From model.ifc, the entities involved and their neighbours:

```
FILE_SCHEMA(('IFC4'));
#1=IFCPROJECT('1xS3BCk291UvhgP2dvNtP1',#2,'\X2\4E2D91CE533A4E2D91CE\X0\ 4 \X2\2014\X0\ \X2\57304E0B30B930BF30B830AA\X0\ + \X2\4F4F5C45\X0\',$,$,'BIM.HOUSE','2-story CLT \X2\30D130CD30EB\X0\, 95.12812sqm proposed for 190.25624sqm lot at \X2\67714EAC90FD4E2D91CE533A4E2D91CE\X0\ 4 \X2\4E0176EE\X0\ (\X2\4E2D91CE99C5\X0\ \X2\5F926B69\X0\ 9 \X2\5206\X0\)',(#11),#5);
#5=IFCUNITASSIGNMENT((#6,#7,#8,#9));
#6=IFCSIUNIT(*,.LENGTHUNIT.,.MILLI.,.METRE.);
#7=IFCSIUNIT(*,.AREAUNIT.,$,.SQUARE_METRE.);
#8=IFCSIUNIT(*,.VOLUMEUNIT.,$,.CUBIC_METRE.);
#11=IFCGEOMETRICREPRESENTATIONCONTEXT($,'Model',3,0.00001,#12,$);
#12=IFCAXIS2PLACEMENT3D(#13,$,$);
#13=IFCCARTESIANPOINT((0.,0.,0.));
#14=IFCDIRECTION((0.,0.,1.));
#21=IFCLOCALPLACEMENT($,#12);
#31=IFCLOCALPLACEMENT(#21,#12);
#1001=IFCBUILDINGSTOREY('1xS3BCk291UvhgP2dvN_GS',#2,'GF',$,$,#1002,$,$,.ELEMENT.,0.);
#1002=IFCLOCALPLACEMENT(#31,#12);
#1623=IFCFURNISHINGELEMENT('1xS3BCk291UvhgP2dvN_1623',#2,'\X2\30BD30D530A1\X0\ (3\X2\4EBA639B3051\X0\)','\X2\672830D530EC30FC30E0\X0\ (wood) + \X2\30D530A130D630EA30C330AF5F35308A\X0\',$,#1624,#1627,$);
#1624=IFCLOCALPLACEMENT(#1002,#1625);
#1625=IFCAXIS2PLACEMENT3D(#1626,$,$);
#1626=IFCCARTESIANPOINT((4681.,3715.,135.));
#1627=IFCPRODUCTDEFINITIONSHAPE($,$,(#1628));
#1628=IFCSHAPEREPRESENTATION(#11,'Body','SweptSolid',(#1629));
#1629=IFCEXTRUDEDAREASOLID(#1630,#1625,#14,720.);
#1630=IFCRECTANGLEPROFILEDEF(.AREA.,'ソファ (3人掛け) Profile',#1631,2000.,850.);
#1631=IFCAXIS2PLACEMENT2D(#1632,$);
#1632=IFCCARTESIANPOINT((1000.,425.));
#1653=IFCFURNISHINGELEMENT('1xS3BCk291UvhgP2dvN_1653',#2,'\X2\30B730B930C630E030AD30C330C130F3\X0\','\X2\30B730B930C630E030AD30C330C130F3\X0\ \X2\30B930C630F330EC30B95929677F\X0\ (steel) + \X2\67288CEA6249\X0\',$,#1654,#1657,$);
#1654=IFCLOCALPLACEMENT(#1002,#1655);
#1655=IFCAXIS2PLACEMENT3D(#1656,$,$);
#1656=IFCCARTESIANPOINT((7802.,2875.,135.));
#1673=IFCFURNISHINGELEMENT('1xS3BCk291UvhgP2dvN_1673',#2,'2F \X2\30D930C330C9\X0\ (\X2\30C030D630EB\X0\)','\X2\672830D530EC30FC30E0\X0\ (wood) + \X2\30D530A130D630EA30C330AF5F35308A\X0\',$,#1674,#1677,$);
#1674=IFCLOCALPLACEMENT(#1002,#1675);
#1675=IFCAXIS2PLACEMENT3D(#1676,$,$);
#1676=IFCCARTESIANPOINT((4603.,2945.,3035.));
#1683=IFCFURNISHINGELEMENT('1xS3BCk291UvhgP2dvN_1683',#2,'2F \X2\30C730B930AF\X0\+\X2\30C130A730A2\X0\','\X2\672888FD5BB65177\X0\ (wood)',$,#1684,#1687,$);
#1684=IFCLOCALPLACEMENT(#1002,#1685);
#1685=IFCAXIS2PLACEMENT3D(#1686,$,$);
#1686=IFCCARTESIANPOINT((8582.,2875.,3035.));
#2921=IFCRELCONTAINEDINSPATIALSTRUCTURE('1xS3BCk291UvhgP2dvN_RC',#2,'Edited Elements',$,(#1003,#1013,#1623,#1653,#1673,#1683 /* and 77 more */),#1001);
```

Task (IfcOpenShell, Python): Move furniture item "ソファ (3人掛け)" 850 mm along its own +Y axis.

```python
import ifcopenshell
import ifcopenshell.api.geometry
import ifcopenshell.util.placement
import ifcopenshell.util.unit

model = ifcopenshell.open("model.ifc")
unit_scale = ifcopenshell.util.unit.calculate_unit_scale(model)

item = model.by_id(1623)
matrix = ifcopenshell.util.placement.get_local_placement(item.ObjectPlacement)
matrix[:3, 3] += matrix[:3, 1] * 0.85 / unit_scale
ifcopenshell.api.geometry.edit_object_placement(model, product=item, matrix=matrix, is_si=False)

print(ifcopenshell.util.placement.get_local_placement(item.ObjectPlacement).round(3) + 0.0)

model.write("model_v2.ifc")
```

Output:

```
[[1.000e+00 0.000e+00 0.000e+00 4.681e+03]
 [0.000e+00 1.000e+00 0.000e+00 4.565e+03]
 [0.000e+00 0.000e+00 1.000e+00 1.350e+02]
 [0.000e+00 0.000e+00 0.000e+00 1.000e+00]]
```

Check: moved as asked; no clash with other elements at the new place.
